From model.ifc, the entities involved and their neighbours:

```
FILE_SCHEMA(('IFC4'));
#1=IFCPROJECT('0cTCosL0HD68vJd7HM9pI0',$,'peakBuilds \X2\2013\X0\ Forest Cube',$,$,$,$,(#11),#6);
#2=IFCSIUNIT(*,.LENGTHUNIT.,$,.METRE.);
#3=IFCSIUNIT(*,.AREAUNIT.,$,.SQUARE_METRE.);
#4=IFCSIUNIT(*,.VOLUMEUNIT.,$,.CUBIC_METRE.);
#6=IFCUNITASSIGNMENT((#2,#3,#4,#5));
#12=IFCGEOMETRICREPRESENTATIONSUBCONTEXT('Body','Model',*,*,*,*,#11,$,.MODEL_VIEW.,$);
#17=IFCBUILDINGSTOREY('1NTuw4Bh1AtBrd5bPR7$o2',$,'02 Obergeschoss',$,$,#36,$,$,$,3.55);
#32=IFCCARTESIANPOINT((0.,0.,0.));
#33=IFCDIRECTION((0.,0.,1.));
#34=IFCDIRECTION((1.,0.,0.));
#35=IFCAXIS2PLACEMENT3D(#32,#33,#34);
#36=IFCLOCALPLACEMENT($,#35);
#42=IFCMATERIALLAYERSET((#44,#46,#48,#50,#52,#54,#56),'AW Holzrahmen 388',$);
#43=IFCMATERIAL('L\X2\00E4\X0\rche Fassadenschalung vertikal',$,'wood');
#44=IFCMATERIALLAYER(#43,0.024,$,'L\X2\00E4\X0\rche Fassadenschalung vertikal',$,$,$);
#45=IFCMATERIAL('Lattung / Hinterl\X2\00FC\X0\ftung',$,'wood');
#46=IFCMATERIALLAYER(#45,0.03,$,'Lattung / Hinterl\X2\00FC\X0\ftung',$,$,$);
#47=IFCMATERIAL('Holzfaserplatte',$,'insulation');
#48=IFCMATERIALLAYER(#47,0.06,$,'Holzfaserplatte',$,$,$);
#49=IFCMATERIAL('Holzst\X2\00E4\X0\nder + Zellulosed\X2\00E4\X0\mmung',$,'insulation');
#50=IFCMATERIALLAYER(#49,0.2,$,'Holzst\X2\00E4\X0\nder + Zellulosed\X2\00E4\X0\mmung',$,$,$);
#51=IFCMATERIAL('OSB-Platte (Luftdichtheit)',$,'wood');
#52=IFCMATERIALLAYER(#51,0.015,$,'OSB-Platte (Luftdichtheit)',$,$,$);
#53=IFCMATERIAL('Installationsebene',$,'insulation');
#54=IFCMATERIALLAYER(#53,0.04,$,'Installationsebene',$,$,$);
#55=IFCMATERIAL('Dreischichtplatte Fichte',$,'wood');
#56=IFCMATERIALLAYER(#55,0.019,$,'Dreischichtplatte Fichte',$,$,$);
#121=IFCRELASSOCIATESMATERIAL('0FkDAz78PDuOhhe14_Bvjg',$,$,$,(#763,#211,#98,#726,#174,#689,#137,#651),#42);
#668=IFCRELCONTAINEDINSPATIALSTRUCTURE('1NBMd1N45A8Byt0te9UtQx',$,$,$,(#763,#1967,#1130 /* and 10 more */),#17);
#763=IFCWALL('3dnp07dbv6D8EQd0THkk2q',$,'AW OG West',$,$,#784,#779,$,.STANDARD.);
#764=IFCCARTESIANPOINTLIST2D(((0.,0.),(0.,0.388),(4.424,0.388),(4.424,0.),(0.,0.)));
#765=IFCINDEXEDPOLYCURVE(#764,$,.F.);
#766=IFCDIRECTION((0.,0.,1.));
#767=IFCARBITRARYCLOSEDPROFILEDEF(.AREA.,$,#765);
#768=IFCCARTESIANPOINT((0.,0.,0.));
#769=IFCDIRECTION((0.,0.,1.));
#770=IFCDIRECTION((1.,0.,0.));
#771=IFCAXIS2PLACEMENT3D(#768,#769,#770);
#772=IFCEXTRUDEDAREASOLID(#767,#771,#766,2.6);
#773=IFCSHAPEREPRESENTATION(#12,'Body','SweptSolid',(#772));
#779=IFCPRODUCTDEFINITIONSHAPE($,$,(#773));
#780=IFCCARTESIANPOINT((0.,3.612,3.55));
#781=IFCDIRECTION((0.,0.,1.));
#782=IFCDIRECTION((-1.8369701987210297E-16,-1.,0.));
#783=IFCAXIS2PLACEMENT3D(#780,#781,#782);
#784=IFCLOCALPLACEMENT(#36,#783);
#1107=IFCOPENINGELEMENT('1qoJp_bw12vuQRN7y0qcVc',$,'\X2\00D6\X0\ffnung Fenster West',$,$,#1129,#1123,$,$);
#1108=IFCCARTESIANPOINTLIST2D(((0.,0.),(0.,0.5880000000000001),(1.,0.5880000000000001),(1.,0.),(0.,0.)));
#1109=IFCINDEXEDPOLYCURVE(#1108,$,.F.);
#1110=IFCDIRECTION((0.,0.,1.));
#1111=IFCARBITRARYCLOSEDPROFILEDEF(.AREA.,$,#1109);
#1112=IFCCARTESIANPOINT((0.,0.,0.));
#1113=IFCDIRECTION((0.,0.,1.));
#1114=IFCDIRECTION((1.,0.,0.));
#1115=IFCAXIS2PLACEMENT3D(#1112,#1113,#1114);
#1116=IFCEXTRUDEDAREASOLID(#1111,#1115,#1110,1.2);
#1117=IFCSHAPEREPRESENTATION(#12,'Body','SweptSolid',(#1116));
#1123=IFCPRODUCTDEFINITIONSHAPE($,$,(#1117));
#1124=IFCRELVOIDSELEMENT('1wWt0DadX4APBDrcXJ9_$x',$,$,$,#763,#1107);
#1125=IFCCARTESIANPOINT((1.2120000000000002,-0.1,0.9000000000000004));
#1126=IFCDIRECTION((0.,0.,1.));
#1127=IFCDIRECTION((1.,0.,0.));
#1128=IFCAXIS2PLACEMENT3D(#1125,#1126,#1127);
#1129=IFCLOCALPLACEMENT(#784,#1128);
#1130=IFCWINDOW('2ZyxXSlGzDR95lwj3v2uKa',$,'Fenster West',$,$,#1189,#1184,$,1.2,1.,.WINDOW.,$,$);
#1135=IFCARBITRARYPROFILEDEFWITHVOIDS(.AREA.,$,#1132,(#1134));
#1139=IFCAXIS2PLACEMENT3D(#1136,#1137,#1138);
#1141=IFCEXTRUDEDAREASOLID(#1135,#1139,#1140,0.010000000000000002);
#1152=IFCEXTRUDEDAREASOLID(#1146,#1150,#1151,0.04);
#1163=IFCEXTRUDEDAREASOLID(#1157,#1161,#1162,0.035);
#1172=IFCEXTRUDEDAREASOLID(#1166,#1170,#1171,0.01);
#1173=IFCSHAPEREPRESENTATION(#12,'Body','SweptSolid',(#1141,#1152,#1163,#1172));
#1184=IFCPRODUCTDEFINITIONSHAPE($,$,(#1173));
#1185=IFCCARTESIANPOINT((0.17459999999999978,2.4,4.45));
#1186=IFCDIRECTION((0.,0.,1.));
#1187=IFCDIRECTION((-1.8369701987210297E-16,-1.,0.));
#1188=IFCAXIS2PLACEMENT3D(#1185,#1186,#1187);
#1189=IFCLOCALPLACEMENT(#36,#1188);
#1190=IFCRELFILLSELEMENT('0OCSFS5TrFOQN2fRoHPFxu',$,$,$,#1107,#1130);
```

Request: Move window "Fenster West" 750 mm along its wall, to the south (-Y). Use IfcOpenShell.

```python
import ifcopenshell
import ifcopenshell.api.geometry
import ifcopenshell.util.placement
import ifcopenshell.util.unit

model = ifcopenshell.open("model.ifc")
unit_scale = ifcopenshell.util.unit.calculate_unit_scale(model)

window = model.by_id(1130)
opening = window.FillsVoids[0].RelatingOpeningElement
wall = opening.VoidsElements[0].RelatingBuildingElement

wall_matrix = ifcopenshell.util.placement.get_local_placement(wall.ObjectPlacement)
shift = wall_matrix[:3, 0] * 0.75 / unit_scale
before = ifcopenshell.util.placement.get_local_placement(window.ObjectPlacement)[:3, 3].copy()

# The window is not placed relative to its opening, so move both.
for product in (opening, window):
    matrix = ifcopenshell.util.placement.get_local_placement(product.ObjectPlacement)
    matrix[:3, 3] += shift
    ifcopenshell.api.geometry.edit_object_placement(model, product=product, matrix=matrix, is_si=False)

after = ifcopenshell.util.placement.get_local_placement(window.ObjectPlacement)[:3, 3]
print("window moved by", (after - before).round(3) + 0.0)

model.write("model_v2.ifc")
```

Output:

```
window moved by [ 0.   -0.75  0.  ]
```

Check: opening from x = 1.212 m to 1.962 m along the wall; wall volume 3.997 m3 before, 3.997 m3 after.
